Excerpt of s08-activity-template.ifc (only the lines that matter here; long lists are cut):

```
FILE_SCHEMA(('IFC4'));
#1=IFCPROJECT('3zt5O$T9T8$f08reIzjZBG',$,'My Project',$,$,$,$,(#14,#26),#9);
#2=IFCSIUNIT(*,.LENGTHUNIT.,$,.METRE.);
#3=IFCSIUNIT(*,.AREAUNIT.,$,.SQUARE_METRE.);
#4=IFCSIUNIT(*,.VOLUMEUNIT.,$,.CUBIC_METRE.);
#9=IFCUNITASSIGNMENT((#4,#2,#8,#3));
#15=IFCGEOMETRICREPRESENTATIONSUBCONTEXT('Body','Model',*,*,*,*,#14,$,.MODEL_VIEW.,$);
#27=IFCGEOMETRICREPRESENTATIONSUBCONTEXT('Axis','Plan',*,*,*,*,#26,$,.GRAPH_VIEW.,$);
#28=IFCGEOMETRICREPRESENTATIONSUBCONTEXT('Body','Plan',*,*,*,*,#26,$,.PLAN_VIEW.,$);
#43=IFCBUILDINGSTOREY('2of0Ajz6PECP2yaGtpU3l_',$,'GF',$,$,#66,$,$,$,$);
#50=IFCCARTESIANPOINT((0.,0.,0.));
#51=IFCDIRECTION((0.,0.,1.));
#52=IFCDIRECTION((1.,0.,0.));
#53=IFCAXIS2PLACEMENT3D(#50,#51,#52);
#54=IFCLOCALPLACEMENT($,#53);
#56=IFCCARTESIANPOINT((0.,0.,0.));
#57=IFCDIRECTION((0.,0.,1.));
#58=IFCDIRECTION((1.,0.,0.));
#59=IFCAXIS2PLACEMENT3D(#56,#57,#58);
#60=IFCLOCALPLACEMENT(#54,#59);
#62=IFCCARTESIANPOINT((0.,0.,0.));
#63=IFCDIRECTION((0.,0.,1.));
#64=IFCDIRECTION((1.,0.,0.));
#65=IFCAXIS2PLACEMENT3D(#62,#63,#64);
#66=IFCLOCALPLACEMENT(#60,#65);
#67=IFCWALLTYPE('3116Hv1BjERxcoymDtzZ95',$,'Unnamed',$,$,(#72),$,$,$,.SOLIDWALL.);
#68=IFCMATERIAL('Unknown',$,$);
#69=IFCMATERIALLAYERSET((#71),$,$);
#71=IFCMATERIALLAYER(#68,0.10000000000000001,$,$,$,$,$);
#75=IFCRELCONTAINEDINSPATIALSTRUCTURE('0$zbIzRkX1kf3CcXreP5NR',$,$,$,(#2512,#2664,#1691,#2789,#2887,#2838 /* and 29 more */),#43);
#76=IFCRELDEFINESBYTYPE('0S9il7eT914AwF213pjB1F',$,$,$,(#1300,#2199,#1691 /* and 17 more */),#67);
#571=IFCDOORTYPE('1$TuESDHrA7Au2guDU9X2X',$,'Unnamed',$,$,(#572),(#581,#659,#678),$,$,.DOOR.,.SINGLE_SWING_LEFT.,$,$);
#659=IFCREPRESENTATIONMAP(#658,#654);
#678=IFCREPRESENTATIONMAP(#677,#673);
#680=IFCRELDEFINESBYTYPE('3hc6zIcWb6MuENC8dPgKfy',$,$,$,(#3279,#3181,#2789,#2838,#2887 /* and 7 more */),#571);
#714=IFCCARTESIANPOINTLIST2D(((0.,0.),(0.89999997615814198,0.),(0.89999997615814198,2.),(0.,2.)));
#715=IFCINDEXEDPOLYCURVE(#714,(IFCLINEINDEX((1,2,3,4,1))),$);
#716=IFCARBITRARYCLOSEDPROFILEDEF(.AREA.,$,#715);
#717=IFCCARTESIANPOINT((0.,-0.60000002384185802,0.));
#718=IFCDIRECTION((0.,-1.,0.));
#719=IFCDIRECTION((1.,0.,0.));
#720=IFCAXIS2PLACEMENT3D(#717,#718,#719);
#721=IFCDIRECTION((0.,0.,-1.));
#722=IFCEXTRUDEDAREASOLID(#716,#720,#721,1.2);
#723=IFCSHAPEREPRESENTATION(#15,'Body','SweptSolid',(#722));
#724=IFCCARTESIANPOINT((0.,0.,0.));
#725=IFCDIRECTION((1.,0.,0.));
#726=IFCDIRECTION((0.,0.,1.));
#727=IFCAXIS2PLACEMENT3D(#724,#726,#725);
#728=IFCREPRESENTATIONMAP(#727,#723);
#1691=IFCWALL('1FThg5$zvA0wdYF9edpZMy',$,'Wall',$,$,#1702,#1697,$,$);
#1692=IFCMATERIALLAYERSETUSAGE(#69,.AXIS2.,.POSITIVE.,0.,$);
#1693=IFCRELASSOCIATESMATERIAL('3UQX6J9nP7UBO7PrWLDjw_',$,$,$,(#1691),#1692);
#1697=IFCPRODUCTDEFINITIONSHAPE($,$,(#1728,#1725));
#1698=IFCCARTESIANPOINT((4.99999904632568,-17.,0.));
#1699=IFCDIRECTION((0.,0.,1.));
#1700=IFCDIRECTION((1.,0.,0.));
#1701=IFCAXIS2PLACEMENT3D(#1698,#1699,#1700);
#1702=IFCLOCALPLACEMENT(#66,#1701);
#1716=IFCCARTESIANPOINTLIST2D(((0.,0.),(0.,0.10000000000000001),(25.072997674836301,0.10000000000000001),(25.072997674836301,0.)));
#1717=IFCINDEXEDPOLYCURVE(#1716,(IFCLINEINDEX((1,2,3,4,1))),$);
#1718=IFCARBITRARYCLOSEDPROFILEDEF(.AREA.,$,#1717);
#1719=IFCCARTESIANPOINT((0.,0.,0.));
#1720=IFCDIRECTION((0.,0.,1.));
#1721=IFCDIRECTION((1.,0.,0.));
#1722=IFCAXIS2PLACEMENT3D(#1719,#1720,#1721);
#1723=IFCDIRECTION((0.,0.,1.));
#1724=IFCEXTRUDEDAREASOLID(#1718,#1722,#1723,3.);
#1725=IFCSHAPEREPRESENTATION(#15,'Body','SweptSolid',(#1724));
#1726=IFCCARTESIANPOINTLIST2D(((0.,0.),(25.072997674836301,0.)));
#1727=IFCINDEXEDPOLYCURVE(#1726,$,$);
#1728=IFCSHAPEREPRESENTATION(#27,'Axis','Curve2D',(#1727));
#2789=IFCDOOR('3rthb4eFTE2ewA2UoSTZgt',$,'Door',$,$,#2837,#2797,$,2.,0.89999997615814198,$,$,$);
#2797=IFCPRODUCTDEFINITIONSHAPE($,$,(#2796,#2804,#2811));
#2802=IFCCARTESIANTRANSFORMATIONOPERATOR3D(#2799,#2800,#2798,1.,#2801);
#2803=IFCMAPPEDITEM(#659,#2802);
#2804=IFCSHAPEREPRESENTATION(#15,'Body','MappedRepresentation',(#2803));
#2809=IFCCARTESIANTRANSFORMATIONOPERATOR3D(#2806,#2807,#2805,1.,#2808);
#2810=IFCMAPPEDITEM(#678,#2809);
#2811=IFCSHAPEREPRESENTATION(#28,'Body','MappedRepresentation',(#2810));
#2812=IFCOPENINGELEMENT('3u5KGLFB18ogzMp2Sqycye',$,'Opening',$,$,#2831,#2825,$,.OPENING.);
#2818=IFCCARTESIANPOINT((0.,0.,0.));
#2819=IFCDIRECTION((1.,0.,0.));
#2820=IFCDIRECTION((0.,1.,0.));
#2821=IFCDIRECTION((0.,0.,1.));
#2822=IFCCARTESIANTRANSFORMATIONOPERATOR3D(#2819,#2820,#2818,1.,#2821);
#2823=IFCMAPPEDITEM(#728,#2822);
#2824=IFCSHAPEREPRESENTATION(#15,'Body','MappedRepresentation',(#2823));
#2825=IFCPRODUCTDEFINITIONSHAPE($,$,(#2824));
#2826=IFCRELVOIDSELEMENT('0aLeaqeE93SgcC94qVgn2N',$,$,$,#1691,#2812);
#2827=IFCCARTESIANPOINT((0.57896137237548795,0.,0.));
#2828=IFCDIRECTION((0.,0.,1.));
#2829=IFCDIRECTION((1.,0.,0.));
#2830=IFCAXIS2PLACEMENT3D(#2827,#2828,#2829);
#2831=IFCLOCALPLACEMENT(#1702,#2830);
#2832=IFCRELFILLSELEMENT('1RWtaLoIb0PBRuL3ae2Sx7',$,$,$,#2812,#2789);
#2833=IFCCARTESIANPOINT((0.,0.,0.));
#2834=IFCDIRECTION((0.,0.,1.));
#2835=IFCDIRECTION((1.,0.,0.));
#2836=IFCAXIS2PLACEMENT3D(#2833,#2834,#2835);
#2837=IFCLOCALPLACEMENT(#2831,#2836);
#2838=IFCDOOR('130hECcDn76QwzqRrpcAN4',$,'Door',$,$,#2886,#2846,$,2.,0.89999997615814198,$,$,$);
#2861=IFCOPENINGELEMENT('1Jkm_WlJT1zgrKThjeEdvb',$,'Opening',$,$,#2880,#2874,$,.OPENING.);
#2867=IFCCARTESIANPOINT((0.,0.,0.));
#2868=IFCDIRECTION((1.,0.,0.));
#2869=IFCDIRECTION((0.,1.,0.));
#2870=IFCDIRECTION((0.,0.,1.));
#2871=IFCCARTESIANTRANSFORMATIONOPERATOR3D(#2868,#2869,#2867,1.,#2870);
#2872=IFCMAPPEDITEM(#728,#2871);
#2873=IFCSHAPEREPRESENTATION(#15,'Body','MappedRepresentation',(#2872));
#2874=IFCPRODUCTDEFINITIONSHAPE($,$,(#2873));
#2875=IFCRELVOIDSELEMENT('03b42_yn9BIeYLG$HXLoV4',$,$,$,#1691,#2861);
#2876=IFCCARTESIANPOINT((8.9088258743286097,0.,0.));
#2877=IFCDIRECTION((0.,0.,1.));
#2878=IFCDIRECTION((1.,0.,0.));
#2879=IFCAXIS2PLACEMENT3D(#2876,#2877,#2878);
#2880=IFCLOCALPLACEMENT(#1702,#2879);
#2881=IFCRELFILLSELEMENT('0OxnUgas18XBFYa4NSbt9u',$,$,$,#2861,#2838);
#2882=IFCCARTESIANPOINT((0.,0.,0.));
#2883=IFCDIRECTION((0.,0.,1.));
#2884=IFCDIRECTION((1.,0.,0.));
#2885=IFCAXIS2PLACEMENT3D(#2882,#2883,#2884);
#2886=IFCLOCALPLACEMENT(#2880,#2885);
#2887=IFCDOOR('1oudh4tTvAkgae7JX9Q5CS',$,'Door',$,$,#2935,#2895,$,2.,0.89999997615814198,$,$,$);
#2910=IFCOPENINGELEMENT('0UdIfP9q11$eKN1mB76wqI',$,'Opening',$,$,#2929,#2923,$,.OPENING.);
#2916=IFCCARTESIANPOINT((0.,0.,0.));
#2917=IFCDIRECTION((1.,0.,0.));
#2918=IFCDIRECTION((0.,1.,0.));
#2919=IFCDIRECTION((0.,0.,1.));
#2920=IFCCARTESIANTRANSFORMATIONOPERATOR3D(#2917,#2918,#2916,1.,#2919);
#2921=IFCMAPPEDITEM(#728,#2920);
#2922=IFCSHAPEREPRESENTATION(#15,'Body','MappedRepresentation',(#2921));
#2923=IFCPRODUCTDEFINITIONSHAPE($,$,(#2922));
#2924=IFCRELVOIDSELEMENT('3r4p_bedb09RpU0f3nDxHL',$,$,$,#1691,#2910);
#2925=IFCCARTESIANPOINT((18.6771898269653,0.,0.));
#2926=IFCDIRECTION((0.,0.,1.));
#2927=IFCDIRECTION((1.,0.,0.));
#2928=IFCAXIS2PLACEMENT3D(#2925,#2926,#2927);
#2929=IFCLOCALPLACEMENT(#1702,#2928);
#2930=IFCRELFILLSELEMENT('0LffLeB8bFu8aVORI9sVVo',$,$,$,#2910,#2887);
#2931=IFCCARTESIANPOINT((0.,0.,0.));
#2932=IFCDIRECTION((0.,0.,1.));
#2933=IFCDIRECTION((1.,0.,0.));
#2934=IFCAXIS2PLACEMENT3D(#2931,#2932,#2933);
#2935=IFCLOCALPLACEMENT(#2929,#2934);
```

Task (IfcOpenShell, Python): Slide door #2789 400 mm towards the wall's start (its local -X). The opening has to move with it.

```python
import ifcopenshell
import ifcopenshell.api.geometry
import ifcopenshell.util.placement
import ifcopenshell.util.unit

model = ifcopenshell.open("s08-activity-template.ifc")
unit_scale = ifcopenshell.util.unit.calculate_unit_scale(model)

door = model.by_id(2789)
opening = door.FillsVoids[0].RelatingOpeningElement
wall = opening.VoidsElements[0].RelatingBuildingElement

wall_matrix = ifcopenshell.util.placement.get_local_placement(wall.ObjectPlacement)
shift = wall_matrix[:3, 0] * -0.4 / unit_scale
before = ifcopenshell.util.placement.get_local_placement(door.ObjectPlacement)[:3, 3].copy()

# The door is placed relative to its opening, so it follows when the opening moves.
matrix = ifcopenshell.util.placement.get_local_placement(opening.ObjectPlacement)
matrix[:3, 3] += shift
ifcopenshell.api.geometry.edit_object_placement(
    model, product=opening, matrix=matrix, is_si=False, should_transform_children=True
)

after = ifcopenshell.util.placement.get_local_placement(door.ObjectPlacement)[:3, 3]
print("door moved by", (after - before).round(3) + 0.0)

model.write("s08-activity-template_rev.ifc")
```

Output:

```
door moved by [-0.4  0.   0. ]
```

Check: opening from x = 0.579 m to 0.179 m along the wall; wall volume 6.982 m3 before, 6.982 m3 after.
